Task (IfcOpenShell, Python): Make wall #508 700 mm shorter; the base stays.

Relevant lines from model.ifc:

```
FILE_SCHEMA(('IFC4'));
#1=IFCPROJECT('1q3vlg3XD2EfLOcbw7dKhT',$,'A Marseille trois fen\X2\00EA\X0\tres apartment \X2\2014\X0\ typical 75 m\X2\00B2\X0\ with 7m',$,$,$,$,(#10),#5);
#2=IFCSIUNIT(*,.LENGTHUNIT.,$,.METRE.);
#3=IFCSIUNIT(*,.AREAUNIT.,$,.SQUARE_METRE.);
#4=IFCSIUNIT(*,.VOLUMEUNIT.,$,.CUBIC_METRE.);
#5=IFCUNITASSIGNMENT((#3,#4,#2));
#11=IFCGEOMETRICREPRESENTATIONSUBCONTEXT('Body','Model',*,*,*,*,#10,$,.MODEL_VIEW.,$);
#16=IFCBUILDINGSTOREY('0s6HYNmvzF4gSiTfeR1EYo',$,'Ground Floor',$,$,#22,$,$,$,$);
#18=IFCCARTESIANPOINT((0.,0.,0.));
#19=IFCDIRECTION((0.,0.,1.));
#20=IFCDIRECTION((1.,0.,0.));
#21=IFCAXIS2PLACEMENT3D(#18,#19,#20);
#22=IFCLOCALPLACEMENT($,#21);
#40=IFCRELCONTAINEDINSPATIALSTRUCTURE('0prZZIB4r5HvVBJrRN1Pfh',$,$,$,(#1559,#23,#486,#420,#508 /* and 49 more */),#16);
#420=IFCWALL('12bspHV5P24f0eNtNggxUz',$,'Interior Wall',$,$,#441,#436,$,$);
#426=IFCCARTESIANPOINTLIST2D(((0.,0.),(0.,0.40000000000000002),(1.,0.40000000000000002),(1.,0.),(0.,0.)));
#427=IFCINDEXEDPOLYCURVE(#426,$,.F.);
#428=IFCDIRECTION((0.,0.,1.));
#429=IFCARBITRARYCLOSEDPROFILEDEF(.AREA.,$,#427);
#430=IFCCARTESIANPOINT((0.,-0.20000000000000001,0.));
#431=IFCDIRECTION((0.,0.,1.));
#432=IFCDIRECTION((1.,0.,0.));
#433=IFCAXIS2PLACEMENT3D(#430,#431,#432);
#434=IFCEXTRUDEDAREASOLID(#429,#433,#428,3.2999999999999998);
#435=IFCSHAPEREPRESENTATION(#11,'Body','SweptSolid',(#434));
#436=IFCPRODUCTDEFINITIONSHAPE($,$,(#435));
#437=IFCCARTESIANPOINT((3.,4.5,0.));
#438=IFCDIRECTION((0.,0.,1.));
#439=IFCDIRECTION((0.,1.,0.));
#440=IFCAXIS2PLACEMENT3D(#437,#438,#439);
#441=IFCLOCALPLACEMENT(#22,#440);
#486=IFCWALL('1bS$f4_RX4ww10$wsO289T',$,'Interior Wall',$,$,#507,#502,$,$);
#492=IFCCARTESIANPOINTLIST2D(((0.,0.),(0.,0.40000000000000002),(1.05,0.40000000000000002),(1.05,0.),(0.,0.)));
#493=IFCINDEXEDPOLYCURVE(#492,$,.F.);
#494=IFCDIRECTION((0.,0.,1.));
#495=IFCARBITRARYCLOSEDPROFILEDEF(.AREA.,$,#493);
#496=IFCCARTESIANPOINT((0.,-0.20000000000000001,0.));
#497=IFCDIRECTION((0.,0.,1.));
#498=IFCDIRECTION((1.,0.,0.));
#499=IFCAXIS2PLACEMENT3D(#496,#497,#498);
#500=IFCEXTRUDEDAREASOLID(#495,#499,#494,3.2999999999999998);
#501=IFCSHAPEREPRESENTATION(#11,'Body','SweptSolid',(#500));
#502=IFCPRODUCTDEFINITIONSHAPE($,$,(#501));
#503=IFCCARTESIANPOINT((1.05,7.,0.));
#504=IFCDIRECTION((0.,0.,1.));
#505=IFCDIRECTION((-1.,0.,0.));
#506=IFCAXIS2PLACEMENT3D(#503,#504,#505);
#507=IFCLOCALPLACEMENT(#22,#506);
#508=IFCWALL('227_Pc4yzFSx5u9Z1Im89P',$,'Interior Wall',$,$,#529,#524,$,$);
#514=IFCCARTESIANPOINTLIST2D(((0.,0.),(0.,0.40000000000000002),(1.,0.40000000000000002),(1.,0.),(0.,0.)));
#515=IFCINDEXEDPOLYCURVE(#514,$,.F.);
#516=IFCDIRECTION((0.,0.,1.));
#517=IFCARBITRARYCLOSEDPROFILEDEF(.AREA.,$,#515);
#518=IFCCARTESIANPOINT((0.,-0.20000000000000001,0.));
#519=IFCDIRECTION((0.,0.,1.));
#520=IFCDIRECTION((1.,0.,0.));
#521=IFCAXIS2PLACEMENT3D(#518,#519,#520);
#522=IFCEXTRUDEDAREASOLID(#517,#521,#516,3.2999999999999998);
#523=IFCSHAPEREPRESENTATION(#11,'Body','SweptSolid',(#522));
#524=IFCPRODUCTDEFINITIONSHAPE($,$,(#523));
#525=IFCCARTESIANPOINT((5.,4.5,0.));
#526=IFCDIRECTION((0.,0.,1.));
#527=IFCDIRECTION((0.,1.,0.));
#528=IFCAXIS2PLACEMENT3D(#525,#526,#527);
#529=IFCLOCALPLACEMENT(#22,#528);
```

```python
import ifcopenshell
import ifcopenshell.geom
import ifcopenshell.util.representation
import ifcopenshell.util.shape
import ifcopenshell.util.unit

model = ifcopenshell.open("model.ifc")
unit_scale = ifcopenshell.util.unit.calculate_unit_scale(model)
settings = ifcopenshell.geom.settings()


def volume(element):
    """Net volume in cubic metres, openings subtracted."""
    shape = ifcopenshell.geom.create_shape(settings, element)
    return ifcopenshell.util.shape.get_volume(shape.geometry)


wall = model.by_guid("227_Pc4yzFSx5u9Z1Im89P")
before = volume(wall)

body = ifcopenshell.util.representation.get_representation(wall, "Model", "Body")
solid = body.Items[0]
old_height = solid.Depth
solid.Depth -= 0.7 / unit_scale
after = volume(wall)

print(f"height {old_height:g} -> {solid.Depth:g}, volume {before:.3f} -> {after:.3f} m3")

model.write("model_edited.ifc")
```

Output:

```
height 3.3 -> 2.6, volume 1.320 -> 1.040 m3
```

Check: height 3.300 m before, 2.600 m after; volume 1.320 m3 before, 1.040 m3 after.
